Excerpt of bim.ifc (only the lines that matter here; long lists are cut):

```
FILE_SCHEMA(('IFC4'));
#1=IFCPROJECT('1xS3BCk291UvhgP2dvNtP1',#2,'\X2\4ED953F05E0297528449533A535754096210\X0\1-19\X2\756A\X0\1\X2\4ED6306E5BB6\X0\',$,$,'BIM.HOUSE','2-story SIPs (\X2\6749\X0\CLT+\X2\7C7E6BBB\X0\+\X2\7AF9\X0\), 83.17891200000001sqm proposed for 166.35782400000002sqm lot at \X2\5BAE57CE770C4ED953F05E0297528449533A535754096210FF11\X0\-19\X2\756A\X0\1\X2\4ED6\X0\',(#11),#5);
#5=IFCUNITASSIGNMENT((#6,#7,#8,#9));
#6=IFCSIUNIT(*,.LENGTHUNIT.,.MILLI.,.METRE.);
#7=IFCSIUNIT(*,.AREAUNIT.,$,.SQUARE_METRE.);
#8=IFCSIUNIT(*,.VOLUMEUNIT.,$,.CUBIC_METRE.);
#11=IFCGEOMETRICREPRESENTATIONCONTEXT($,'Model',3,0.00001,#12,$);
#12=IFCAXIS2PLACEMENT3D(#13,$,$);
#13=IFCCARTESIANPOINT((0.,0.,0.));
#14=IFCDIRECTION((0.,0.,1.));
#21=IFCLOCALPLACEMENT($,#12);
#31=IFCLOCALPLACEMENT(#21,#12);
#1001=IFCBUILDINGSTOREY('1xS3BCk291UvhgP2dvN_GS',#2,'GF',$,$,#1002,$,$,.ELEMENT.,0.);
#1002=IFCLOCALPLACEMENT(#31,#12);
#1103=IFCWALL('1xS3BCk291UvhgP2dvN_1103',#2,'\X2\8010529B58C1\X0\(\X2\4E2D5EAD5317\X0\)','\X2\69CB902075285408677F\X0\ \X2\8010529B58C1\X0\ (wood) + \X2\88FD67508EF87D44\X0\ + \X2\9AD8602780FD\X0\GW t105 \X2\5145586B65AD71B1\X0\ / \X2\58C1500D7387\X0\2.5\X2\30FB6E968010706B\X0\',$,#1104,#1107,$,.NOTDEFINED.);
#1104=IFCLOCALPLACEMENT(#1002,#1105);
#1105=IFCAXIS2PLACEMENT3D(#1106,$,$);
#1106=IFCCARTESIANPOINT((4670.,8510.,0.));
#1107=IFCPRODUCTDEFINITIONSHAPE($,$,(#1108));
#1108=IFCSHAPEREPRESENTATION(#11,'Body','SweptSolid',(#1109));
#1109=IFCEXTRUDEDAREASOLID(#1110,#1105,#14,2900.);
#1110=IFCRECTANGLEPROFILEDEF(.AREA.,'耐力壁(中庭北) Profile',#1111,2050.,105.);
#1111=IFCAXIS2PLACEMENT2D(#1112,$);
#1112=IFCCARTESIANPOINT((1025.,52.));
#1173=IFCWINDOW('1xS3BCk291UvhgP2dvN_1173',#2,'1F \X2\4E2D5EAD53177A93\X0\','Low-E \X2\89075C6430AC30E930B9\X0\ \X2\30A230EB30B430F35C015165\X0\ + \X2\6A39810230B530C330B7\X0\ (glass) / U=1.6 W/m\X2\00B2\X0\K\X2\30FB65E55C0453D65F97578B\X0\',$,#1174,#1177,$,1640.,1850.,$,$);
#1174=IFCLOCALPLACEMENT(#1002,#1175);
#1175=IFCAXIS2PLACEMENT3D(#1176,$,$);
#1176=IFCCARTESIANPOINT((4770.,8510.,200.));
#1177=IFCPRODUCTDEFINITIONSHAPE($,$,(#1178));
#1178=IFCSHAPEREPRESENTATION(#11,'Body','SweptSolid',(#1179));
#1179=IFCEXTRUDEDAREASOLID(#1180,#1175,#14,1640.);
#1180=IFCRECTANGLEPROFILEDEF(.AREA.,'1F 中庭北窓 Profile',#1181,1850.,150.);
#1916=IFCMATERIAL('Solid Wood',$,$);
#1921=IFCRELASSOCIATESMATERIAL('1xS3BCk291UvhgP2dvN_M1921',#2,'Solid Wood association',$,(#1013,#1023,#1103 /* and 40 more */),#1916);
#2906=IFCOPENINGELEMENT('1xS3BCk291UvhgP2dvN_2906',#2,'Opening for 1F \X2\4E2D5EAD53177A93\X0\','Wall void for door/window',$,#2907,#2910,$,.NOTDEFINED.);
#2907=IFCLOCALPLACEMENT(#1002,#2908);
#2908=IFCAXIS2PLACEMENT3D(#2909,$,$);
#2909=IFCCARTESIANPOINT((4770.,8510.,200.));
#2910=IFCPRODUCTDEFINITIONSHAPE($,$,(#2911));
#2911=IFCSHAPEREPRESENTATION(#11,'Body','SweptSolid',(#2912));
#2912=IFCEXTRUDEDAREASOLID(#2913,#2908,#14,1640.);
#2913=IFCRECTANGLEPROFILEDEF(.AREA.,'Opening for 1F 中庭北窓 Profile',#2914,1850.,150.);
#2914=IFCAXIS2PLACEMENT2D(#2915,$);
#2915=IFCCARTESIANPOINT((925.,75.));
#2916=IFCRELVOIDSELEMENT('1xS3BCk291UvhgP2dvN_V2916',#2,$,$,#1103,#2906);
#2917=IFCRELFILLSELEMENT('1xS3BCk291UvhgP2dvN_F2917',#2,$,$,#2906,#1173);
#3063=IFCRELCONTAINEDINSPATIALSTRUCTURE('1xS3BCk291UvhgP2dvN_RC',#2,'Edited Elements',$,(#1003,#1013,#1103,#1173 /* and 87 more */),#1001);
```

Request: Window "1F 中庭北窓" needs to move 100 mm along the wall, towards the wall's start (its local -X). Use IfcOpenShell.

```python
import ifcopenshell
import ifcopenshell.api.geometry
import ifcopenshell.util.placement
import ifcopenshell.util.unit

model = ifcopenshell.open("bim.ifc")
unit_scale = ifcopenshell.util.unit.calculate_unit_scale(model)

window = model.by_guid("1xS3BCk291UvhgP2dvN_1173")
opening = window.FillsVoids[0].RelatingOpeningElement
wall = opening.VoidsElements[0].RelatingBuildingElement

wall_matrix = ifcopenshell.util.placement.get_local_placement(wall.ObjectPlacement)
shift = wall_matrix[:3, 0] * -0.1 / unit_scale
before = ifcopenshell.util.placement.get_local_placement(window.ObjectPlacement)[:3, 3].copy()

# The window is not placed relative to its opening, so move both.
for product in (opening, window):
    matrix = ifcopenshell.util.placement.get_local_placement(product.ObjectPlacement)
    matrix[:3, 3] += shift
    ifcopenshell.api.geometry.edit_object_placement(model, product=product, matrix=matrix, is_si=False)

after = ifcopenshell.util.placement.get_local_placement(window.ObjectPlacement)[:3, 3]
print("window moved by", (after - before).round(3) + 0.0)

model.write("bim_v2.ifc")
```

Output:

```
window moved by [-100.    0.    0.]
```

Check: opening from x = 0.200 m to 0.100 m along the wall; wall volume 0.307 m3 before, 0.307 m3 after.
